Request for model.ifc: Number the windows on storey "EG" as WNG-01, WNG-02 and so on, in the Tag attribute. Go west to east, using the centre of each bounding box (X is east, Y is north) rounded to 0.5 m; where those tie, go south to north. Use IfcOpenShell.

First a look at what the model holds.

```python
import ifcopenshell
import ifcopenshell.util.element
import ifcopenshell.util.placement

model = ifcopenshell.open("model.ifc")
print(model.schema)
storey = next(s for s in model.by_type("IfcBuildingStorey") if s.Name == "EG")
windows = [e for e in ifcopenshell.util.element.get_decomposition(storey) if e.is_a("IfcWindow")]
for e in sorted(windows, key=lambda e: e.id()):
    origin = ifcopenshell.util.placement.get_local_placement(e.ObjectPlacement)[:3, 3]
    print(e.id(), e.Tag, e.Name, origin.round(2) + 0.0, sep=" | ")
```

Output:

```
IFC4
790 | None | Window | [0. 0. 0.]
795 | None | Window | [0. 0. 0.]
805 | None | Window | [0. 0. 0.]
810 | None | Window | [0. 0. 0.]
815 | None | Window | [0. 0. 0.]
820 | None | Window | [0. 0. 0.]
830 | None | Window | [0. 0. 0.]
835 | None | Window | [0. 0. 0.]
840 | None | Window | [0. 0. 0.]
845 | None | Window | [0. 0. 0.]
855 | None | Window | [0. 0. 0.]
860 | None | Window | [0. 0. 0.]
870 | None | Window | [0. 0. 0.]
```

```python
import ifcopenshell
import ifcopenshell.geom
import ifcopenshell.util.element
import ifcopenshell.util.shape

model = ifcopenshell.open("model.ifc")
settings = ifcopenshell.geom.settings()
settings.set("use-world-coords", True)


def centre(element):
    shape = ifcopenshell.geom.create_shape(settings, element)
    return ifcopenshell.util.shape.get_bbox_centroid(shape.geometry)


storey = next(s for s in model.by_type("IfcBuildingStorey") if s.Name == "EG")
windows = [e for e in ifcopenshell.util.element.get_decomposition(storey) if e.is_a("IfcWindow")]

# Insertion points can sit at a corner or the storey origin, so sort by the geometry (in metres).
centres = {e: centre(e) for e in windows}
windows.sort(key=lambda e: (round(centres[e][0] / 0.5), centres[e][1]))

for i, e in enumerate(windows, start=1):
    number = f"WNG-{i:02d}"
    e.Tag = number
    print(e.id(), number)

model.write("model_edited.ifc")
```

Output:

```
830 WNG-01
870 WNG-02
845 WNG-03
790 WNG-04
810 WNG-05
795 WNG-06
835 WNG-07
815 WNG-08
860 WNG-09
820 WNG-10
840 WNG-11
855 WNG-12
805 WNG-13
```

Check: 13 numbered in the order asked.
